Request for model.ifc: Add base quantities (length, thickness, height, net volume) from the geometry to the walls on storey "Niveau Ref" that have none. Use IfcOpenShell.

First a look at what the model holds.

```python
import ifcopenshell
import ifcopenshell.util.element
import ifcopenshell.util.unit

model = ifcopenshell.open("model.ifc")
print(model.schema)
for unit_type in ("LENGTHUNIT", "AREAUNIT", "VOLUMEUNIT"):
    print(unit_type, ifcopenshell.util.unit.calculate_unit_scale(model, unit_type))
storey = next(s for s in model.by_type("IfcBuildingStorey") if s.Name == "Niveau Ref")
walls = [e for e in ifcopenshell.util.element.get_decomposition(storey) if e.is_a("IfcWall")]
for e in sorted(walls, key=lambda e: e.id()):
    print(e.id(), e.is_a(), e.Name, list(ifcopenshell.util.element.get_psets(e, qtos_only=True)), sep=" | ")
```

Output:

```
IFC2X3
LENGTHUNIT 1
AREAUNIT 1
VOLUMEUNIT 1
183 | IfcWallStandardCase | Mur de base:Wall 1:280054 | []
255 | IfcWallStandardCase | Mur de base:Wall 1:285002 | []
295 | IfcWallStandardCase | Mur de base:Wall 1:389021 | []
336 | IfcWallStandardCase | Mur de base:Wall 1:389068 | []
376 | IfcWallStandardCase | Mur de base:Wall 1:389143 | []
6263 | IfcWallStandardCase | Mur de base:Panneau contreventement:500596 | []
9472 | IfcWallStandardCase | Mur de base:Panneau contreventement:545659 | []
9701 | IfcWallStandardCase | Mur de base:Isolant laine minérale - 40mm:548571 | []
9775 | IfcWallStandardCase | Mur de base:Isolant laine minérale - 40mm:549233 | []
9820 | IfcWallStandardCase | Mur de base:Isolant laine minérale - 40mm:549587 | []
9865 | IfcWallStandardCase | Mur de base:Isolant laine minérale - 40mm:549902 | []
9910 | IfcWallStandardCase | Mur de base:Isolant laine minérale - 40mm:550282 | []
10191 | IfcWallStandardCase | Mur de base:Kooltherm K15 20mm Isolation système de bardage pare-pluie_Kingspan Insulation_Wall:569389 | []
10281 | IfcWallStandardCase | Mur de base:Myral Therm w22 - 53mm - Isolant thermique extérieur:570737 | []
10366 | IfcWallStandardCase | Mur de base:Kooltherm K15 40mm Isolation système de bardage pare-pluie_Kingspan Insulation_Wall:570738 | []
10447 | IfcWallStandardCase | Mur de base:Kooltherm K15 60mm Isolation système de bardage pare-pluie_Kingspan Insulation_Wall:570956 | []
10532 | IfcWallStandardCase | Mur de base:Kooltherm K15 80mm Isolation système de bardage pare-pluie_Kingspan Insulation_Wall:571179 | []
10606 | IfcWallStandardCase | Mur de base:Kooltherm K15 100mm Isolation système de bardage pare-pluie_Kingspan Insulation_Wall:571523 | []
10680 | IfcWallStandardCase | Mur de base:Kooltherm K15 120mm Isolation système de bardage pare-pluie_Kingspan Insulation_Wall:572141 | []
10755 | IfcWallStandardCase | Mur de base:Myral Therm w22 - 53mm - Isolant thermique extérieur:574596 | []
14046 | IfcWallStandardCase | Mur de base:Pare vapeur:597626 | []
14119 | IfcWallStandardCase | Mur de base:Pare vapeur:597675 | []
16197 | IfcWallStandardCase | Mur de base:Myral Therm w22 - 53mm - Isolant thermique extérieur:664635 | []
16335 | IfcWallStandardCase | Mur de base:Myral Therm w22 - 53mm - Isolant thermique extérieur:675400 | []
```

```python
import ifcopenshell
import ifcopenshell.api.pset
import ifcopenshell.geom
import ifcopenshell.util.element
import ifcopenshell.util.shape
import ifcopenshell.util.unit

model = ifcopenshell.open("model.ifc")
unit_scale = ifcopenshell.util.unit.calculate_unit_scale(model)
volume_scale = ifcopenshell.util.unit.calculate_unit_scale(model, "VOLUMEUNIT")
settings = ifcopenshell.geom.settings()

storey = next(s for s in model.by_type("IfcBuildingStorey") if s.Name == "Niveau Ref")
walls = [e for e in ifcopenshell.util.element.get_decomposition(storey) if e.is_a("IfcWall")]

for e in sorted(walls, key=lambda e: e.id()):
    if ifcopenshell.util.element.get_psets(e, qtos_only=True, should_inherit=False):
        continue
    # Geometry comes back in metres, in the element's own axes.
    shape = ifcopenshell.geom.create_shape(settings, e)
    values = {
        "Length": ifcopenshell.util.shape.get_x(shape.geometry) / unit_scale,
        "Width": ifcopenshell.util.shape.get_y(shape.geometry) / unit_scale,
        "Height": ifcopenshell.util.shape.get_z(shape.geometry) / unit_scale,
        "NetVolume": ifcopenshell.util.shape.get_volume(shape.geometry) / volume_scale,
    }
    qto = ifcopenshell.api.pset.add_qto(model, product=e, name="BaseQuantities")
    ifcopenshell.api.pset.edit_qto(model, qto=qto, properties=values)
    print(e.id(), {k: round(v, 3) for k, v in values.items()})

model.write("model_rev.ifc")
```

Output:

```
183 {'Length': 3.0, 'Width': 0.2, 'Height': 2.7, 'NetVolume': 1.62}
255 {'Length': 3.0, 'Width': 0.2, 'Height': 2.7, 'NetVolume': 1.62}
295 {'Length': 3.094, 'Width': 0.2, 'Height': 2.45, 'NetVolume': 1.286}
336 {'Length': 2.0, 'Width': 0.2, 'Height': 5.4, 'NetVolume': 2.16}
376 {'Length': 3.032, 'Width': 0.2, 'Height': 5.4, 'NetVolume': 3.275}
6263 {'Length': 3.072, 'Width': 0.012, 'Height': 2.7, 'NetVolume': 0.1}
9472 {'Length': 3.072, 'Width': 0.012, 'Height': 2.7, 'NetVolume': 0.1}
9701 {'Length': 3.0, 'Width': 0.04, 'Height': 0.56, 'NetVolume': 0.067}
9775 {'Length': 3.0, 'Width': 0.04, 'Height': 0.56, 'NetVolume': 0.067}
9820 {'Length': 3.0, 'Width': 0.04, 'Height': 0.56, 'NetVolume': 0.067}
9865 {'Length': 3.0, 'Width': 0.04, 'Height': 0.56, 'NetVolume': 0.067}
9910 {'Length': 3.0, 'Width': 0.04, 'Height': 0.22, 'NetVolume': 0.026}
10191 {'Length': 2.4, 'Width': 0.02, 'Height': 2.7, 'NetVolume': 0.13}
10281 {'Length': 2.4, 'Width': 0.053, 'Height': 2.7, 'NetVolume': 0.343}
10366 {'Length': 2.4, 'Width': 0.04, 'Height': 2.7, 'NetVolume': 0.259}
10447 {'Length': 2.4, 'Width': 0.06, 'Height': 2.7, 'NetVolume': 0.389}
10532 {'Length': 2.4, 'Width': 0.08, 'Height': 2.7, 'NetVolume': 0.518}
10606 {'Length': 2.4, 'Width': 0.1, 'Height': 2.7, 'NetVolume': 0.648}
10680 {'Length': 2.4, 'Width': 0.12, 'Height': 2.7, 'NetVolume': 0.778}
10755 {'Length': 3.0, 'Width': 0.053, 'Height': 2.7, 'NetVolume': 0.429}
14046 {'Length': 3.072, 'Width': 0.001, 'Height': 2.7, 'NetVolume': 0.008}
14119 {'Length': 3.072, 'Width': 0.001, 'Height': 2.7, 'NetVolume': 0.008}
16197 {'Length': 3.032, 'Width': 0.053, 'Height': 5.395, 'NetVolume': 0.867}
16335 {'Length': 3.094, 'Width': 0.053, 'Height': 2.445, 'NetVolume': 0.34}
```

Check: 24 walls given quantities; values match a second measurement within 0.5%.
